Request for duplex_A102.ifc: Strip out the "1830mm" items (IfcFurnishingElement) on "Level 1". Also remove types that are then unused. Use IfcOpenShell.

First a look at what the model holds.

```python
import ifcopenshell
import ifcopenshell.util.element

model = ifcopenshell.open("duplex_A102.ifc")
print(model.schema)
storey = next(s for s in model.by_type("IfcBuildingStorey") if s.Name == "Level 1")
furniture = [e for e in ifcopenshell.util.element.get_decomposition(storey) if e.is_a("IfcFurnishingElement")]
seen = {}
for e in furniture:
    element_type = ifcopenshell.util.element.get_type(e)
    name = element_type.Name if element_type not in (None, e) else None
    seen[name] = seen.get(name, 0) + 1
for name, count in sorted(seen.items(), key=str):
    print(count, "x", name)
```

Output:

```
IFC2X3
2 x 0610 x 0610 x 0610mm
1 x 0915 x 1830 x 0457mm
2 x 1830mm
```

```python
import ifcopenshell
import ifcopenshell.api.root
import ifcopenshell.util.element

model = ifcopenshell.open("duplex_A102.ifc")

storey = next(s for s in model.by_type("IfcBuildingStorey") if s.Name == "Level 1")
furniture = [e for e in ifcopenshell.util.element.get_decomposition(storey) if e.is_a("IfcFurnishingElement")]
targets = [e for e in furniture if (t := ifcopenshell.util.element.get_type(e)) not in (None, e) and t.Name == "1830mm"]
types = {ifcopenshell.util.element.get_type(e) for e in targets} - {None, *targets}

for e in targets:
    ifcopenshell.api.root.remove_product(model, product=e)
print(len(targets), "removed")

unused = [t for t in types if not ifcopenshell.util.element.get_types(t)]
for t in unused:
    ifcopenshell.api.root.remove_product(model, product=t)
print(len(unused), "unused types removed")

model.write("duplex_A102_updated.ifc")
```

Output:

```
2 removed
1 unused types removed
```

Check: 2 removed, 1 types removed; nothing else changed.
